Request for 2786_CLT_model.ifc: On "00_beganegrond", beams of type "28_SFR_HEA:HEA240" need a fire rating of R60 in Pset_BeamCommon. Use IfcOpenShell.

First a look at what the model holds.

```python
import ifcopenshell
import ifcopenshell.util.element

model = ifcopenshell.open("2786_CLT_model.ifc")
print(model.schema)
storey = next(s for s in model.by_type("IfcBuildingStorey") if s.Name == "00_beganegrond")
beams = [e for e in ifcopenshell.util.element.get_decomposition(storey) if e.is_a("IfcBeam")]
seen = {}
for e in beams:
    element_type = ifcopenshell.util.element.get_type(e)
    key = (element_type.Name if element_type != e and element_type else None, ifcopenshell.util.element.get_pset(e, "Pset_BeamCommon", "FireRating"))
    seen[key] = seen.get(key, 0) + 1
for (name, value), count in sorted(seen.items(), key=str):
    print(count, "x", name, "|", value)
```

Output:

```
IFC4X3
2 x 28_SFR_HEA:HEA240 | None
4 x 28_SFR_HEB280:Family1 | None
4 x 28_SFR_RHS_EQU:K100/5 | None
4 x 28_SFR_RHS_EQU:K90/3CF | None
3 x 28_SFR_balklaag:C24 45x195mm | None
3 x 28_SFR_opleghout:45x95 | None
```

```python
import ifcopenshell
import ifcopenshell.api.pset
import ifcopenshell.util.element

model = ifcopenshell.open("2786_CLT_model.ifc")

storey = next(s for s in model.by_type("IfcBuildingStorey") if s.Name == "00_beganegrond")
beams = [e for e in ifcopenshell.util.element.get_decomposition(storey) if e.is_a("IfcBeam")]

count = 0
for e in beams:
    element_type = ifcopenshell.util.element.get_type(e)
    if element_type in (None, e) or element_type.Name != "28_SFR_HEA:HEA240":
        continue
    # add_pset returns the element's existing set when there is one.
    pset = ifcopenshell.api.pset.add_pset(model, product=e, name="Pset_BeamCommon")
    ifcopenshell.api.pset.edit_pset(model, pset=pset, properties={"FireRating": "R60"})
    count += 1

print(count, "beams updated")

model.write("2786_CLT_model_v2.ifc")
```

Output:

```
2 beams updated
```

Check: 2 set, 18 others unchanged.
